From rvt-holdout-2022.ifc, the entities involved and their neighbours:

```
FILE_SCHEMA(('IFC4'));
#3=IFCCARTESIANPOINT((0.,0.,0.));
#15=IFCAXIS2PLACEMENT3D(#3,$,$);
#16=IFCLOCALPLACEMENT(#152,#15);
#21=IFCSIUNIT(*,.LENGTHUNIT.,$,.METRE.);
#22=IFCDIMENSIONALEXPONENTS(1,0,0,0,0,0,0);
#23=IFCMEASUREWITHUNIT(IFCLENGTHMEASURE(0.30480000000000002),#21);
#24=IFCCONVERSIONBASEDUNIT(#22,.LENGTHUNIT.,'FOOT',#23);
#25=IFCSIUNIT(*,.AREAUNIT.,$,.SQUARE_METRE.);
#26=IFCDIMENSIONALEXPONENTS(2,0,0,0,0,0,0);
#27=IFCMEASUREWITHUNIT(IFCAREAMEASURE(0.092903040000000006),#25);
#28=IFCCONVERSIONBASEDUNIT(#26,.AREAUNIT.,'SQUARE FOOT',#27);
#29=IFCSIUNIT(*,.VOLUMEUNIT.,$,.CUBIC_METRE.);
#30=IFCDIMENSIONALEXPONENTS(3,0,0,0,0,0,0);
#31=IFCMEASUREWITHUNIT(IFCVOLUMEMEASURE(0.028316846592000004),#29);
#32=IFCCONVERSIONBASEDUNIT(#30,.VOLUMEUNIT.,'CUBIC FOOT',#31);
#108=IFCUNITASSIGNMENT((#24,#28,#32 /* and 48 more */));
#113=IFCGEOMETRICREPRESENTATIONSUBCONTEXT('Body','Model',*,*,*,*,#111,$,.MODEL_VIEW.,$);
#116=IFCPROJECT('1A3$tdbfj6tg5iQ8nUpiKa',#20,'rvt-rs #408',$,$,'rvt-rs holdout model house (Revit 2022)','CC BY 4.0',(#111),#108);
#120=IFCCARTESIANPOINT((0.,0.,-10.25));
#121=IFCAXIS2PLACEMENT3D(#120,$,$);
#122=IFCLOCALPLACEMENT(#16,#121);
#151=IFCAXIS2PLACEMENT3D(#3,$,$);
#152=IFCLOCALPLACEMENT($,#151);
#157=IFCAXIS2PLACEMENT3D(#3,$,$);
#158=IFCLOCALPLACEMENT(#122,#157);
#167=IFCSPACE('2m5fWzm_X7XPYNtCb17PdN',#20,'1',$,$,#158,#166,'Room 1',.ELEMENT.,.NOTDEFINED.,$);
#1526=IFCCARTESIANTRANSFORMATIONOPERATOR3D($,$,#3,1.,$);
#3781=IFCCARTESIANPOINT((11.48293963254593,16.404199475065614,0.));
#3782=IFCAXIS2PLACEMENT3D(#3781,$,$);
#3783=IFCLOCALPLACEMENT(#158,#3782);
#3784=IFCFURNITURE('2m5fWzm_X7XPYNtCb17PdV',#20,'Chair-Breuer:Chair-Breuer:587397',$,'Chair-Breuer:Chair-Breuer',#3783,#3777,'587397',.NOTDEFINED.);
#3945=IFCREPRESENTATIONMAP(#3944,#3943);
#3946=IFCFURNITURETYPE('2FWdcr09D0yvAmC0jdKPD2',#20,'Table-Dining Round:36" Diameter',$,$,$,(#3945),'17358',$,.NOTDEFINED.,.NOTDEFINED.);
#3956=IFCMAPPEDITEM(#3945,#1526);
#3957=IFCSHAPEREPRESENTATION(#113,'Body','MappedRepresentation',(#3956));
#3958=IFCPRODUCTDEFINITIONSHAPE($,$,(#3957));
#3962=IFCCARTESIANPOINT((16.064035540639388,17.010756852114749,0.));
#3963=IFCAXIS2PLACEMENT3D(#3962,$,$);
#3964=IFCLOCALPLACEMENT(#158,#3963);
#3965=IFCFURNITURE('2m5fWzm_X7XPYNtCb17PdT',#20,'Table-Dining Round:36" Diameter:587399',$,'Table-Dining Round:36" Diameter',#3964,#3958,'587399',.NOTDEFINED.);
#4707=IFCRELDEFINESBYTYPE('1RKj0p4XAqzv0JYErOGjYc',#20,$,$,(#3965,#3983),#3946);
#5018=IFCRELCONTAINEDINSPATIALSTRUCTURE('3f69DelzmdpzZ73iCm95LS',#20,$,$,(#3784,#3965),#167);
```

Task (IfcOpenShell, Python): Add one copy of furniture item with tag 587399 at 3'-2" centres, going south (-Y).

```python
import numpy as np
import ifcopenshell
import ifcopenshell.api.geometry
import ifcopenshell.api.root
import ifcopenshell.util.element
import ifcopenshell.util.placement
import ifcopenshell.util.unit

model = ifcopenshell.open("rvt-holdout-2022.ifc")
unit_scale = ifcopenshell.util.unit.calculate_unit_scale(model)


def reuse_history(source, copy):
    """copy_class also copies each property set's owner history, people and application; keep the originals."""
    for rel in copy.IsDefinedBy:
        if rel.is_a("IfcRelDefinesByProperties") and (history := rel.RelatingPropertyDefinition.OwnerHistory):
            rel.RelatingPropertyDefinition.OwnerHistory = source.OwnerHistory
            ifcopenshell.util.element.remove_deep2(model, history)


source = model.by_id(3965)
base = ifcopenshell.util.placement.get_local_placement(source.ObjectPlacement)
step = np.array([0.0, -1.0, 0.0]) * 38 * 0.0254 / unit_scale

for i in range(1, 2):
    copy = ifcopenshell.api.root.copy_class(model, product=source)
    copy.Representation = ifcopenshell.util.element.copy_deep(
        model, source.Representation, exclude=["IfcGeometricRepresentationContext", "IfcRepresentationMap"]
    )
    copy.Name = 'Table-Dining Round:36" Diameter'
    copy.Tag = None
    reuse_history(source, copy)
    matrix = base.copy()
    matrix[:3, 3] += i * step
    print("added at", matrix[:3, 3].round(3) + 0.0)
    ifcopenshell.api.geometry.edit_object_placement(model, product=copy, matrix=matrix, is_si=False)

model.write("rvt-holdout-2022_v2.ifc")
```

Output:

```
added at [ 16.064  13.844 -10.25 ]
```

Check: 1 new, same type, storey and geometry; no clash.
